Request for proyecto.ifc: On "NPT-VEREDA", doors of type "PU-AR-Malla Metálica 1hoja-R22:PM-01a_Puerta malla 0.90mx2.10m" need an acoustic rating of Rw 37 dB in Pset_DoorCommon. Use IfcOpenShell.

First a look at what the model holds.

```python
import ifcopenshell
import ifcopenshell.util.element

model = ifcopenshell.open("proyecto.ifc")
print(model.schema)
storey = next(s for s in model.by_type("IfcBuildingStorey") if s.Name == "NPT-VEREDA")
doors = [e for e in ifcopenshell.util.element.get_decomposition(storey) if e.is_a("IfcDoor")]
seen = {}
for e in doors:
    element_type = ifcopenshell.util.element.get_type(e)
    key = (element_type.Name if element_type != e and element_type else None, ifcopenshell.util.element.get_pset(e, "Pset_DoorCommon", "AcousticRating"))
    seen[key] = seen.get(key, 0) + 1
for (name, value), count in sorted(seen.items(), key=str):
    print(count, "x", name, "|", value)
```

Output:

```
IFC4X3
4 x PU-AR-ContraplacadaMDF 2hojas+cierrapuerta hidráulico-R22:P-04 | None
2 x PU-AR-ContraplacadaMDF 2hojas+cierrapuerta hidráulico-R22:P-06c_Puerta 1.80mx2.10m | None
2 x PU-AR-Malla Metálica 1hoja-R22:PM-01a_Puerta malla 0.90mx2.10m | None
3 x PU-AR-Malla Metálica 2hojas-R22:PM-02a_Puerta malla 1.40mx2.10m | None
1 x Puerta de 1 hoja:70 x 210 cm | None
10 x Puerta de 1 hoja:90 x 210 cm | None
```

```python
import ifcopenshell
import ifcopenshell.api.pset
import ifcopenshell.util.element

model = ifcopenshell.open("proyecto.ifc")

storey = next(s for s in model.by_type("IfcBuildingStorey") if s.Name == "NPT-VEREDA")
doors = [e for e in ifcopenshell.util.element.get_decomposition(storey) if e.is_a("IfcDoor")]

count = 0
for e in doors:
    element_type = ifcopenshell.util.element.get_type(e)
    if element_type in (None, e) or element_type.Name != "PU-AR-Malla Metálica 1hoja-R22:PM-01a_Puerta malla 0.90mx2.10m":
        continue
    # add_pset returns the element's existing set when there is one.
    pset = ifcopenshell.api.pset.add_pset(model, product=e, name="Pset_DoorCommon")
    ifcopenshell.api.pset.edit_pset(model, pset=pset, properties={"AcousticRating": "Rw 37 dB"})
    count += 1

print(count, "doors updated")

model.write("proyecto-out.ifc")
```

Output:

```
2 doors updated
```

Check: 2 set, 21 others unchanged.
